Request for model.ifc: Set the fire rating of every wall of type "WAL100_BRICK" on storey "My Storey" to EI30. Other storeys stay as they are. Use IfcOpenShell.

First a look at what the model holds.

```python
import ifcopenshell
import ifcopenshell.util.element

model = ifcopenshell.open("model.ifc")
print(model.schema)
storey = next(s for s in model.by_type("IfcBuildingStorey") if s.Name == "My Storey")
walls = [e for e in ifcopenshell.util.element.get_decomposition(storey) if e.is_a("IfcWall")]
seen = {}
for e in walls:
    element_type = ifcopenshell.util.element.get_type(e)
    key = (element_type.Name if element_type != e and element_type else None, ifcopenshell.util.element.get_pset(e, "Pset_WallCommon", "FireRating"))
    seen[key] = seen.get(key, 0) + 1
for (name, value), count in sorted(seen.items(), key=str):
    print(count, "x", name, "|", value)
```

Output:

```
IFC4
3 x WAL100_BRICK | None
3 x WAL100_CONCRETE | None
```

```python
import ifcopenshell
import ifcopenshell.api.pset
import ifcopenshell.util.element

model = ifcopenshell.open("model.ifc")

storey = next(s for s in model.by_type("IfcBuildingStorey") if s.Name == "My Storey")
walls = [e for e in ifcopenshell.util.element.get_decomposition(storey) if e.is_a("IfcWall")]

count = 0
for e in walls:
    element_type = ifcopenshell.util.element.get_type(e)
    if element_type in (None, e) or element_type.Name != "WAL100_BRICK":
        continue
    # add_pset returns the element's existing set when there is one.
    pset = ifcopenshell.api.pset.add_pset(model, product=e, name="Pset_WallCommon")
    ifcopenshell.api.pset.edit_pset(model, pset=pset, properties={"FireRating": "EI30"})
    count += 1

print(count, "walls updated")

model.write("model_rev.ifc")
```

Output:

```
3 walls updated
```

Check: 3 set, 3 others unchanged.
